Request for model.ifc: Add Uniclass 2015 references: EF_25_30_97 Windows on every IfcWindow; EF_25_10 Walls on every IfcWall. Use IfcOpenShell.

First a look at what the model holds.

```python
import ifcopenshell

model = ifcopenshell.open("model.ifc")
print(model.schema)
print("classifications:", [c.Name for c in model.by_type("IfcClassification")])
for ifc_class in ("IfcDoor", "IfcRoof", "IfcStair", "IfcWall", "IfcWindow"):
    print(ifc_class, len(model.by_type(ifc_class)))
```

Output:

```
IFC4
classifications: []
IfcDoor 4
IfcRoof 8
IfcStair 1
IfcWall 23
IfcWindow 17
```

```python
import ifcopenshell
import ifcopenshell.api.classification

model = ifcopenshell.open("model.ifc")

system = ifcopenshell.api.classification.add_classification(model, classification="Uniclass 2015")

codes = {
    "IfcWindow": ("EF_25_30_97", "Windows"),
    "IfcWall": ("EF_25_10", "Walls"),
}
for ifc_class, (code, name) in codes.items():
    products = model.by_type(ifc_class)
    ifcopenshell.api.classification.add_reference(
        model, products=products, classification=system, identification=code, name=name
    )
    print(code, len(products))

model.write("model-out.ifc")
```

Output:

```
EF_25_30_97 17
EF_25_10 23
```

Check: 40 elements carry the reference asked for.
